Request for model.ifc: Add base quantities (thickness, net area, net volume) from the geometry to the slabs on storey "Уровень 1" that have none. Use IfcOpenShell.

First a look at what the model holds.

```python
import ifcopenshell
import ifcopenshell.util.element
import ifcopenshell.util.unit

model = ifcopenshell.open("model.ifc")
print(model.schema)
for unit_type in ("LENGTHUNIT", "AREAUNIT", "VOLUMEUNIT"):
    print(unit_type, ifcopenshell.util.unit.calculate_unit_scale(model, unit_type))
storey = next(s for s in model.by_type("IfcBuildingStorey") if s.Name == "Уровень 1")
slabs = [e for e in ifcopenshell.util.element.get_decomposition(storey) if e.is_a("IfcSlab")]
for e in sorted(slabs, key=lambda e: e.id()):
    print(e.id(), e.is_a(), e.Name, list(ifcopenshell.util.element.get_psets(e, qtos_only=True)), sep=" | ")
```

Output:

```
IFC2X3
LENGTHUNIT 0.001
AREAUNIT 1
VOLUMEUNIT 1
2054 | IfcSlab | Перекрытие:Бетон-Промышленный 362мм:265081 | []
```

```python
import ifcopenshell
import ifcopenshell.api.pset
import ifcopenshell.geom
import ifcopenshell.util.element
import ifcopenshell.util.shape
import ifcopenshell.util.unit

model = ifcopenshell.open("model.ifc")
unit_scale = ifcopenshell.util.unit.calculate_unit_scale(model)
area_scale = ifcopenshell.util.unit.calculate_unit_scale(model, "AREAUNIT")
volume_scale = ifcopenshell.util.unit.calculate_unit_scale(model, "VOLUMEUNIT")
settings = ifcopenshell.geom.settings()

storey = next(s for s in model.by_type("IfcBuildingStorey") if s.Name == "Уровень 1")
slabs = [e for e in ifcopenshell.util.element.get_decomposition(storey) if e.is_a("IfcSlab")]

for e in sorted(slabs, key=lambda e: e.id()):
    if ifcopenshell.util.element.get_psets(e, qtos_only=True, should_inherit=False):
        continue
    # Geometry comes back in metres, in the element's own axes.
    shape = ifcopenshell.geom.create_shape(settings, e)
    values = {
        "Width": ifcopenshell.util.shape.get_z(shape.geometry) / unit_scale,
        "NetArea": ifcopenshell.util.shape.get_footprint_area(shape.geometry) / area_scale,
        "NetVolume": ifcopenshell.util.shape.get_volume(shape.geometry) / volume_scale,
    }
    qto = ifcopenshell.api.pset.add_qto(model, product=e, name="BaseQuantities")
    ifcopenshell.api.pset.edit_qto(model, qto=qto, properties=values)
    print(e.id(), {k: round(v, 3) for k, v in values.items()})

model.write("model_rev.ifc")
```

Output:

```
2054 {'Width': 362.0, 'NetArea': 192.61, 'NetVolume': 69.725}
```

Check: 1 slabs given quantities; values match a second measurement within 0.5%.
